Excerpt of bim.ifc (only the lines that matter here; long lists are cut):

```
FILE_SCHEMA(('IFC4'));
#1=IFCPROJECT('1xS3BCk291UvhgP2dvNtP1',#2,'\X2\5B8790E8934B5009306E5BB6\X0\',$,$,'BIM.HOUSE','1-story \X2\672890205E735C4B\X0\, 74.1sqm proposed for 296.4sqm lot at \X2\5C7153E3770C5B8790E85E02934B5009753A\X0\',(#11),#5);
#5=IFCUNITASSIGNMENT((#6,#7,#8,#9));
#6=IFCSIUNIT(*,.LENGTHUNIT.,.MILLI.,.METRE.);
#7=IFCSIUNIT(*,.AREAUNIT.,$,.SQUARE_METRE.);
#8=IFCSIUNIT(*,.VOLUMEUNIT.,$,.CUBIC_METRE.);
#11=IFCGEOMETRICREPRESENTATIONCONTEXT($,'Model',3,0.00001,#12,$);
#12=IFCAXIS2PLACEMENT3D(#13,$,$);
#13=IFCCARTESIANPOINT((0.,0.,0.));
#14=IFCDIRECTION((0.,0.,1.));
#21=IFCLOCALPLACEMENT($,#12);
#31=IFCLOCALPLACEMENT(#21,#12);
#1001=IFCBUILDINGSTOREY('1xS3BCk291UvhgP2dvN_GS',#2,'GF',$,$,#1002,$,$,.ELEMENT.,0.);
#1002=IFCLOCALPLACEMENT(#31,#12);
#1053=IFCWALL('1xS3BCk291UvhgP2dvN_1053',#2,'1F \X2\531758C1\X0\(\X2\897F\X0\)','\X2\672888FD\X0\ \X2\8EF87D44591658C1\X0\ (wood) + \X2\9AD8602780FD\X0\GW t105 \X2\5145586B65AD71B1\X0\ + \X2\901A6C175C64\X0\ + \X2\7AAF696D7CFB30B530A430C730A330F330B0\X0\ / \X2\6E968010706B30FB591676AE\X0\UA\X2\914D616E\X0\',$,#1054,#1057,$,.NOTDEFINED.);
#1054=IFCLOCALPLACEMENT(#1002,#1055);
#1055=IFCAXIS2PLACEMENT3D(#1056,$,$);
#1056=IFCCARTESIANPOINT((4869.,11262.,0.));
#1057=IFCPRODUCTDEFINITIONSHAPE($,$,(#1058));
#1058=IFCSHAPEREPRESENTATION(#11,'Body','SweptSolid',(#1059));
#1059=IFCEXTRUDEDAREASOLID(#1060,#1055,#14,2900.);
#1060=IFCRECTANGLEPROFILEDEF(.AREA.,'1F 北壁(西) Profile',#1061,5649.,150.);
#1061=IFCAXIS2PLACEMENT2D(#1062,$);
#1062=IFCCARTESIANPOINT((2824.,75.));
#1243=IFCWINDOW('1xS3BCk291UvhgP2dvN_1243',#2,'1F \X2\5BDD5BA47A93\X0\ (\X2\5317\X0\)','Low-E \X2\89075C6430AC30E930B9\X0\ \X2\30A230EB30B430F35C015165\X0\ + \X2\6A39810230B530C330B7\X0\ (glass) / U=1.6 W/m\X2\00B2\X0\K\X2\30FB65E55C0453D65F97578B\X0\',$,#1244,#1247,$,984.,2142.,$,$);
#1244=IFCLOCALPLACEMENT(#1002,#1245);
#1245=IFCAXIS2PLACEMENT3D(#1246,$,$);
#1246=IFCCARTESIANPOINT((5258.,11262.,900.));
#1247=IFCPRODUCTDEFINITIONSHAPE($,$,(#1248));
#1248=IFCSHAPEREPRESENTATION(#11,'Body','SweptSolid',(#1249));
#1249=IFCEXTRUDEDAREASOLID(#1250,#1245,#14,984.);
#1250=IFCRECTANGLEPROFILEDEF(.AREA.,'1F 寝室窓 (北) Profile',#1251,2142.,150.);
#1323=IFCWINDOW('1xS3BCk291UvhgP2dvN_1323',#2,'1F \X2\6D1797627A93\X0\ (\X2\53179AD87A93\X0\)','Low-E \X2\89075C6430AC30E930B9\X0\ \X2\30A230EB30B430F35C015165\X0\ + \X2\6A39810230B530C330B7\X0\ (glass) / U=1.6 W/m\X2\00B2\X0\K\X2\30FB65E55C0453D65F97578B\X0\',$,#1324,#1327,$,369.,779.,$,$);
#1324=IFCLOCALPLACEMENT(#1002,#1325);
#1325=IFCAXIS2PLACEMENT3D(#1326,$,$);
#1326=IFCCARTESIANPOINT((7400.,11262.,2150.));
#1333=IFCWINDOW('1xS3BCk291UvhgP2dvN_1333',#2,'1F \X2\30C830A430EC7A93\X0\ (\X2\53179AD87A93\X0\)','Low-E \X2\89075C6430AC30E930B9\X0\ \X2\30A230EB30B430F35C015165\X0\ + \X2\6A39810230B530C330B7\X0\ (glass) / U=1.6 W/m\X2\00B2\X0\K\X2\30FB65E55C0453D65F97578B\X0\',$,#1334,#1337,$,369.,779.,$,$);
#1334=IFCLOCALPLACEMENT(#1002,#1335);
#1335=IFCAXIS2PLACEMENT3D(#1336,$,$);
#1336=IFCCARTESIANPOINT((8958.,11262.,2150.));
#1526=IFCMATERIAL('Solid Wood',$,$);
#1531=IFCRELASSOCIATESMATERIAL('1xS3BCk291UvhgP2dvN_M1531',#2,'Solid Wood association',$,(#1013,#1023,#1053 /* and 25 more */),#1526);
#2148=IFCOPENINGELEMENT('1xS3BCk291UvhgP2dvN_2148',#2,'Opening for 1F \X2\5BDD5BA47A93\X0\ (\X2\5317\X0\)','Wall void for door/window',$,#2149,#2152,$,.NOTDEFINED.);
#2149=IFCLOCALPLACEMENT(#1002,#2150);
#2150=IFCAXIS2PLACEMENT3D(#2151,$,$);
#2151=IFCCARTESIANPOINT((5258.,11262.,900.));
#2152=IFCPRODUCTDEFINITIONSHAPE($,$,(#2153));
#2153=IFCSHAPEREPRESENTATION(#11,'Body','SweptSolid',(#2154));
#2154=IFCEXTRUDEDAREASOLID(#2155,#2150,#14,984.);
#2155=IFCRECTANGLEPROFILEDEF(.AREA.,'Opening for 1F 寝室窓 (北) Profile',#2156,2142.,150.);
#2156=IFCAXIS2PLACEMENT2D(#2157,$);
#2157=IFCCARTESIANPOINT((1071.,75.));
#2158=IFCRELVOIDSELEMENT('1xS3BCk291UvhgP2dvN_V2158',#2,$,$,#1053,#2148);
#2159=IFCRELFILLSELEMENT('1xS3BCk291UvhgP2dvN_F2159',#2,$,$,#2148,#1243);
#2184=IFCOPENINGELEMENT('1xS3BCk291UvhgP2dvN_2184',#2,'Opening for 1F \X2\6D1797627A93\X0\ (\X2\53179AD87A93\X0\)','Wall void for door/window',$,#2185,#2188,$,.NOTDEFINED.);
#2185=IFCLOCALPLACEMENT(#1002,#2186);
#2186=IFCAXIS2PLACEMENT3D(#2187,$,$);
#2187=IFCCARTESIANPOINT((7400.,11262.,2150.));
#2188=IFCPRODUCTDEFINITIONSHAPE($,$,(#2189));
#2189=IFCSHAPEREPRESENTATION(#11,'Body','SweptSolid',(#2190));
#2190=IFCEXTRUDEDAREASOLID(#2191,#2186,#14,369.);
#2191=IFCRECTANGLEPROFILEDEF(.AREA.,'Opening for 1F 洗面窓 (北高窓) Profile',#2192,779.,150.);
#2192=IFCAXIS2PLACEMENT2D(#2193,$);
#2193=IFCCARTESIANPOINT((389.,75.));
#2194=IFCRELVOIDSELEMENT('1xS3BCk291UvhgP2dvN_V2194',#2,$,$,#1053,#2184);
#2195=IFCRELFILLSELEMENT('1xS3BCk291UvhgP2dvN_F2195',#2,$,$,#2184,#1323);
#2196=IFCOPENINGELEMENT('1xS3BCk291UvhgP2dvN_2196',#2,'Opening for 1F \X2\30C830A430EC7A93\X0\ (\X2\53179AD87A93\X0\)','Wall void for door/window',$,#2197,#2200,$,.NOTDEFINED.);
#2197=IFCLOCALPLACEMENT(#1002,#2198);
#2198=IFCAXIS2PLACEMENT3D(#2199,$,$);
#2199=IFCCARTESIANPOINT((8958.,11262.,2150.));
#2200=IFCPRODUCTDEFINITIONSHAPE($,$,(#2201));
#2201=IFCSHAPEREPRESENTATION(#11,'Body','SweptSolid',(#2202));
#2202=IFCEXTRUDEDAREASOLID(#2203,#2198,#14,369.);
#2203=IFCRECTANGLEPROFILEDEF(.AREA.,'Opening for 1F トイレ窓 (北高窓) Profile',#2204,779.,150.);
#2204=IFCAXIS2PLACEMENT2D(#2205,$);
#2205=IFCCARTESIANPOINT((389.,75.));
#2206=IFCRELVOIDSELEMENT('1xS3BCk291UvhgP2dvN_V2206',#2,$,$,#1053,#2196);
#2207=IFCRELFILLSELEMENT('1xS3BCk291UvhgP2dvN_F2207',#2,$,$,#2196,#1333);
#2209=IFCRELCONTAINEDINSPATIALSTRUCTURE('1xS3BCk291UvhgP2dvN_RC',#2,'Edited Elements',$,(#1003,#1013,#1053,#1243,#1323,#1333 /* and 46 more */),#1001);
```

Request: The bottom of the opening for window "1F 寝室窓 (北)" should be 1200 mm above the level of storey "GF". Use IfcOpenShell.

```python
import numpy as np
import ifcopenshell
import ifcopenshell.api.geometry
import ifcopenshell.geom
import ifcopenshell.util.element
import ifcopenshell.util.placement
import ifcopenshell.util.shape
import ifcopenshell.util.unit

model = ifcopenshell.open("bim.ifc")
unit_scale = ifcopenshell.util.unit.calculate_unit_scale(model)

window = model.by_id(1243)
opening = window.FillsVoids[0].RelatingOpeningElement
storey = ifcopenshell.util.element.get_container(window, ifc_class="IfcBuildingStorey")
level = ifcopenshell.util.placement.get_local_placement(storey.ObjectPlacement)[2, 3]

# The opening's origin need not be at the sill, so measure its lowest point.
shape = ifcopenshell.geom.create_shape(ifcopenshell.geom.settings(), opening)
bottom = ifcopenshell.util.shape.get_shape_bottom_elevation(shape, shape.geometry) / unit_scale
dz = level + 1.2 / unit_scale - bottom

shift = np.array([0.0, 0.0, dz])
# The window is not placed relative to its opening, so move both.
for product in (opening, window):
    matrix = ifcopenshell.util.placement.get_local_placement(product.ObjectPlacement)
    matrix[:3, 3] += shift
    ifcopenshell.api.geometry.edit_object_placement(model, product=product, matrix=matrix, is_si=False)

print(f"moved by {dz * unit_scale:+.3f} m")

model.write("bim-out.ifc")
```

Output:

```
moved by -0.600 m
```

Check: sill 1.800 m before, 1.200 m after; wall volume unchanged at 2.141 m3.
